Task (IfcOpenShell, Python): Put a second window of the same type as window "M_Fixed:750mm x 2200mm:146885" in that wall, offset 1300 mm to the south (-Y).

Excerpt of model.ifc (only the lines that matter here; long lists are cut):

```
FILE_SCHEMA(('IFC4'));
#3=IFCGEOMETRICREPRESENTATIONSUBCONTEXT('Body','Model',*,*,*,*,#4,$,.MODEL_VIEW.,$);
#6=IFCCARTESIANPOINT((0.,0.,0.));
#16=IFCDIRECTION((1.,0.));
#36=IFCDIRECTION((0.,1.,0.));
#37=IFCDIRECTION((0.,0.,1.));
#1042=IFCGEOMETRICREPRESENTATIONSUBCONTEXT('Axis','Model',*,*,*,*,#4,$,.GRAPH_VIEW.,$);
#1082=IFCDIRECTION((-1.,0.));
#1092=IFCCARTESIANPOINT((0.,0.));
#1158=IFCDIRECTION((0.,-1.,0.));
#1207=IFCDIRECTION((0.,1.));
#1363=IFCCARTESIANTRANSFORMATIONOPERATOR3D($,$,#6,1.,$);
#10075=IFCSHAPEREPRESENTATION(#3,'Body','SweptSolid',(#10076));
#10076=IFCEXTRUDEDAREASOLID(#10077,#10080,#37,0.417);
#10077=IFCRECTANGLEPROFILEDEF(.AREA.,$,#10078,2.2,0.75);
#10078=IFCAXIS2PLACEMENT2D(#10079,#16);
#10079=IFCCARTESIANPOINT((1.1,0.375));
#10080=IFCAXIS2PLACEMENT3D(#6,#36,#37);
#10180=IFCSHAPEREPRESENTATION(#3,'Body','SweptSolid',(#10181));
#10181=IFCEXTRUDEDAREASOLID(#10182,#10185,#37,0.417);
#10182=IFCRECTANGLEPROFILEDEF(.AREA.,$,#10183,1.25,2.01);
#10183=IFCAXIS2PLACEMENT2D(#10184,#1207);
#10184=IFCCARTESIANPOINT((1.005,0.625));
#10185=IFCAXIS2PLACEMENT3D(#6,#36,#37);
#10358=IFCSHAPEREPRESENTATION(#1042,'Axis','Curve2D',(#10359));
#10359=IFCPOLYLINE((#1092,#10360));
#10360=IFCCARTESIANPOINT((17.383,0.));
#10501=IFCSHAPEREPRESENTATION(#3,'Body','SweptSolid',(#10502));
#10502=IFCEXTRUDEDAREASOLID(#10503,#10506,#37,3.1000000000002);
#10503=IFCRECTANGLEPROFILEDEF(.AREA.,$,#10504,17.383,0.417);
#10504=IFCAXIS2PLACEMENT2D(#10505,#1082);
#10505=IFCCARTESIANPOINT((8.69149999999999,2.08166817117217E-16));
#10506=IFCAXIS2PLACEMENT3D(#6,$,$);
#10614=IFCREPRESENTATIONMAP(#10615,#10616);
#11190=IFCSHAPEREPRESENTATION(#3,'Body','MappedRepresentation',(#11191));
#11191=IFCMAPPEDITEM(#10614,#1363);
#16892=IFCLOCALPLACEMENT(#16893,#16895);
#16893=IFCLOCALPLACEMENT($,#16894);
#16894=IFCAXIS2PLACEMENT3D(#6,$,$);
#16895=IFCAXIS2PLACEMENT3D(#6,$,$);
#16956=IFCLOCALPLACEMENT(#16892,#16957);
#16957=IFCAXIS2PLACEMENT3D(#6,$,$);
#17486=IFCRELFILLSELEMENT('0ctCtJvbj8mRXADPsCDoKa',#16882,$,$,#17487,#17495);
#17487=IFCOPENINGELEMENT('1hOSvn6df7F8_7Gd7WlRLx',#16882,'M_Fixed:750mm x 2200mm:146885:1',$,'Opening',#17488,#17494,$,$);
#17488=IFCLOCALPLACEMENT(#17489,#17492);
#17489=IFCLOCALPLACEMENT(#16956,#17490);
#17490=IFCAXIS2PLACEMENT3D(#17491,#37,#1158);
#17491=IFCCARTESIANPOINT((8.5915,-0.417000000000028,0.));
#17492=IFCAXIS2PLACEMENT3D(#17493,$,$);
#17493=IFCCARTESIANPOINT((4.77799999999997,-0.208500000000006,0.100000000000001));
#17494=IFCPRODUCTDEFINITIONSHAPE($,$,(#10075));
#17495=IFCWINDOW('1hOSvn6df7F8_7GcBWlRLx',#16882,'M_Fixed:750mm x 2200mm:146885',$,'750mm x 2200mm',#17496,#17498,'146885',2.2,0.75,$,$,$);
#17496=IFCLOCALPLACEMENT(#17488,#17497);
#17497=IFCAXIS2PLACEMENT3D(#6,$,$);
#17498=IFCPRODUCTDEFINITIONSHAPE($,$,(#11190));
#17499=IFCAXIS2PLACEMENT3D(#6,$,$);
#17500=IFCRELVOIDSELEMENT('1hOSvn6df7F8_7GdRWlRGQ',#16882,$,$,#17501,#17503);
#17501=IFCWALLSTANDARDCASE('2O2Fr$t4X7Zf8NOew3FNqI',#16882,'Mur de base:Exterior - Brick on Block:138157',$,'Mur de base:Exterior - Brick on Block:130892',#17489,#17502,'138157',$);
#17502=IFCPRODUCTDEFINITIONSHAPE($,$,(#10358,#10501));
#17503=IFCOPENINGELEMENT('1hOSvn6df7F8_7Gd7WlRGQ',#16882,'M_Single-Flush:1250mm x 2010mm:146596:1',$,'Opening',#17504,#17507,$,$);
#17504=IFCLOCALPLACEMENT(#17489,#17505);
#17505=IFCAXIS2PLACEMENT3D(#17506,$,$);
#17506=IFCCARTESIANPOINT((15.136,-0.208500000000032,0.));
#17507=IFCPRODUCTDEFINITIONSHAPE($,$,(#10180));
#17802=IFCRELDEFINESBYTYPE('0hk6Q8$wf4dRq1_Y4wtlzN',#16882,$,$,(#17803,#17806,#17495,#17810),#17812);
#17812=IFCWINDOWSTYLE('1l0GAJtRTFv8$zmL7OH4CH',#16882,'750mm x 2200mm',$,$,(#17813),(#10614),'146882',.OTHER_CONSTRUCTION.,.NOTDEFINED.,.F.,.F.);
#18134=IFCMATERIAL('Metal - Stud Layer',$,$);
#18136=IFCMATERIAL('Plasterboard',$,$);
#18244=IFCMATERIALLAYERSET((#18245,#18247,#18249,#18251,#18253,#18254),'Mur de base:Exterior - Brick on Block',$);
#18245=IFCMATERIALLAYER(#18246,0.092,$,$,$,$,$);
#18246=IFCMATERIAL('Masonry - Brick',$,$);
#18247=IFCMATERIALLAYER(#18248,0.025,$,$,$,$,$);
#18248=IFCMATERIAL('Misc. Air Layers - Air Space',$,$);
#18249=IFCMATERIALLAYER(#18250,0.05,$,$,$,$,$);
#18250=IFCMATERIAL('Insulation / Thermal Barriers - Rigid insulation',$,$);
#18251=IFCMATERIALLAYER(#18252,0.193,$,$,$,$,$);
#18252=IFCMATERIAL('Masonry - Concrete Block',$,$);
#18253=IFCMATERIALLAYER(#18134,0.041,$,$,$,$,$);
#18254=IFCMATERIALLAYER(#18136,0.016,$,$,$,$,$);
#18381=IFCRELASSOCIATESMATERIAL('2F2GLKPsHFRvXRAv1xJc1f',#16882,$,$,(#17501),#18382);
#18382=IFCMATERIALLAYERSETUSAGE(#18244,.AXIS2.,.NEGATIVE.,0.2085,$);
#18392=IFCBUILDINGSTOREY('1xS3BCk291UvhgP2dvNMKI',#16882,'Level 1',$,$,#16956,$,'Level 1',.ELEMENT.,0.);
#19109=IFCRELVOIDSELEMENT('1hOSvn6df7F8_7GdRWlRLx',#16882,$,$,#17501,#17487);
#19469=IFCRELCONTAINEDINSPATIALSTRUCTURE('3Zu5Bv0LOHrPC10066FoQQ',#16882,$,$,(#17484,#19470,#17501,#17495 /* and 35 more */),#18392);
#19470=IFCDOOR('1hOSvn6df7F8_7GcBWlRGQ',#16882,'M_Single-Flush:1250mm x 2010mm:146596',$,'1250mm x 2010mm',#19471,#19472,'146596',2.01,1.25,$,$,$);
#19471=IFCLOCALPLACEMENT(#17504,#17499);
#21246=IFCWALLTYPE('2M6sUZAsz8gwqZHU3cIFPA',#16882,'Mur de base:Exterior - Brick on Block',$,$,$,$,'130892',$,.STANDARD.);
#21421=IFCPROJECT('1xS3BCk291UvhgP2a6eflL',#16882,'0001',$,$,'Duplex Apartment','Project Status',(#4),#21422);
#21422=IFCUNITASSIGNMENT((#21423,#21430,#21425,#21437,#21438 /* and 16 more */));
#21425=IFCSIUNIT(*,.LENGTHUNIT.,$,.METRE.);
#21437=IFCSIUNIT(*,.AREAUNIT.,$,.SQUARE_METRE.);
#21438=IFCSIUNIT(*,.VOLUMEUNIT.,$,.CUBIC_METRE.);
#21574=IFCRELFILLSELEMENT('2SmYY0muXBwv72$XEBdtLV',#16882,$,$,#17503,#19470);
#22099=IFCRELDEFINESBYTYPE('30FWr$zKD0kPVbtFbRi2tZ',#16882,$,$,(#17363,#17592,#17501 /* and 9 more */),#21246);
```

```python
import ifcopenshell
import ifcopenshell.api.feature
import ifcopenshell.api.geometry
import ifcopenshell.api.root
import ifcopenshell.geom
import ifcopenshell.util.element
import ifcopenshell.util.placement
import ifcopenshell.util.shape
import ifcopenshell.util.unit

model = ifcopenshell.open("model.ifc")
unit_scale = ifcopenshell.util.unit.calculate_unit_scale(model)
settings = ifcopenshell.geom.settings()


def volume(element):
    """Net volume in cubic metres, openings subtracted."""
    shape = ifcopenshell.geom.create_shape(settings, element)
    return ifcopenshell.util.shape.get_volume(shape.geometry)


def reuse_history(source, copy):
    """copy_class also copies each property set's owner history, people and application; keep the originals."""
    for rel in copy.IsDefinedBy:
        if rel.is_a("IfcRelDefinesByProperties") and (history := rel.RelatingPropertyDefinition.OwnerHistory):
            rel.RelatingPropertyDefinition.OwnerHistory = source.OwnerHistory
            ifcopenshell.util.element.remove_deep2(model, history)


window = model.by_guid("1hOSvn6df7F8_7GcBWlRLx")
opening = window.FillsVoids[0].RelatingOpeningElement
wall = opening.VoidsElements[0].RelatingBuildingElement
before = volume(wall)
shift = ifcopenshell.util.placement.get_local_placement(wall.ObjectPlacement)[:3, 0] * 1.3 / unit_scale

# copy_class copies the void relationship, type, container and properties, but no geometry.
new_opening = ifcopenshell.api.root.copy_class(model, product=opening)
new_opening.Representation = ifcopenshell.util.element.copy_deep(
    model, opening.Representation, exclude=["IfcGeometricRepresentationContext", "IfcRepresentationMap"]
)
new_opening.Name = "M_Fixed:750mm x 2200mm"
new_window = ifcopenshell.api.root.copy_class(model, product=window)
new_window.Representation = ifcopenshell.util.element.copy_deep(
    model, window.Representation, exclude=["IfcGeometricRepresentationContext", "IfcRepresentationMap"]
)
new_window.Name = "M_Fixed:750mm x 2200mm"
new_window.Tag = None
reuse_history(window, new_window)
ifcopenshell.api.feature.add_filling(model, opening=new_opening, element=new_window)

for old, new in ((opening, new_opening), (window, new_window)):
    matrix = ifcopenshell.util.placement.get_local_placement(old.ObjectPlacement)
    matrix[:3, 3] += shift
    ifcopenshell.api.geometry.edit_object_placement(model, product=new, matrix=matrix, is_si=False)

after = volume(wall)

print(f"wall volume {before:.3f} -> {after:.3f} m3")

model.write("model_updated.ifc")
```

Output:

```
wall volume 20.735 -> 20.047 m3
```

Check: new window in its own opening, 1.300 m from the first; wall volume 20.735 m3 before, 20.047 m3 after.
